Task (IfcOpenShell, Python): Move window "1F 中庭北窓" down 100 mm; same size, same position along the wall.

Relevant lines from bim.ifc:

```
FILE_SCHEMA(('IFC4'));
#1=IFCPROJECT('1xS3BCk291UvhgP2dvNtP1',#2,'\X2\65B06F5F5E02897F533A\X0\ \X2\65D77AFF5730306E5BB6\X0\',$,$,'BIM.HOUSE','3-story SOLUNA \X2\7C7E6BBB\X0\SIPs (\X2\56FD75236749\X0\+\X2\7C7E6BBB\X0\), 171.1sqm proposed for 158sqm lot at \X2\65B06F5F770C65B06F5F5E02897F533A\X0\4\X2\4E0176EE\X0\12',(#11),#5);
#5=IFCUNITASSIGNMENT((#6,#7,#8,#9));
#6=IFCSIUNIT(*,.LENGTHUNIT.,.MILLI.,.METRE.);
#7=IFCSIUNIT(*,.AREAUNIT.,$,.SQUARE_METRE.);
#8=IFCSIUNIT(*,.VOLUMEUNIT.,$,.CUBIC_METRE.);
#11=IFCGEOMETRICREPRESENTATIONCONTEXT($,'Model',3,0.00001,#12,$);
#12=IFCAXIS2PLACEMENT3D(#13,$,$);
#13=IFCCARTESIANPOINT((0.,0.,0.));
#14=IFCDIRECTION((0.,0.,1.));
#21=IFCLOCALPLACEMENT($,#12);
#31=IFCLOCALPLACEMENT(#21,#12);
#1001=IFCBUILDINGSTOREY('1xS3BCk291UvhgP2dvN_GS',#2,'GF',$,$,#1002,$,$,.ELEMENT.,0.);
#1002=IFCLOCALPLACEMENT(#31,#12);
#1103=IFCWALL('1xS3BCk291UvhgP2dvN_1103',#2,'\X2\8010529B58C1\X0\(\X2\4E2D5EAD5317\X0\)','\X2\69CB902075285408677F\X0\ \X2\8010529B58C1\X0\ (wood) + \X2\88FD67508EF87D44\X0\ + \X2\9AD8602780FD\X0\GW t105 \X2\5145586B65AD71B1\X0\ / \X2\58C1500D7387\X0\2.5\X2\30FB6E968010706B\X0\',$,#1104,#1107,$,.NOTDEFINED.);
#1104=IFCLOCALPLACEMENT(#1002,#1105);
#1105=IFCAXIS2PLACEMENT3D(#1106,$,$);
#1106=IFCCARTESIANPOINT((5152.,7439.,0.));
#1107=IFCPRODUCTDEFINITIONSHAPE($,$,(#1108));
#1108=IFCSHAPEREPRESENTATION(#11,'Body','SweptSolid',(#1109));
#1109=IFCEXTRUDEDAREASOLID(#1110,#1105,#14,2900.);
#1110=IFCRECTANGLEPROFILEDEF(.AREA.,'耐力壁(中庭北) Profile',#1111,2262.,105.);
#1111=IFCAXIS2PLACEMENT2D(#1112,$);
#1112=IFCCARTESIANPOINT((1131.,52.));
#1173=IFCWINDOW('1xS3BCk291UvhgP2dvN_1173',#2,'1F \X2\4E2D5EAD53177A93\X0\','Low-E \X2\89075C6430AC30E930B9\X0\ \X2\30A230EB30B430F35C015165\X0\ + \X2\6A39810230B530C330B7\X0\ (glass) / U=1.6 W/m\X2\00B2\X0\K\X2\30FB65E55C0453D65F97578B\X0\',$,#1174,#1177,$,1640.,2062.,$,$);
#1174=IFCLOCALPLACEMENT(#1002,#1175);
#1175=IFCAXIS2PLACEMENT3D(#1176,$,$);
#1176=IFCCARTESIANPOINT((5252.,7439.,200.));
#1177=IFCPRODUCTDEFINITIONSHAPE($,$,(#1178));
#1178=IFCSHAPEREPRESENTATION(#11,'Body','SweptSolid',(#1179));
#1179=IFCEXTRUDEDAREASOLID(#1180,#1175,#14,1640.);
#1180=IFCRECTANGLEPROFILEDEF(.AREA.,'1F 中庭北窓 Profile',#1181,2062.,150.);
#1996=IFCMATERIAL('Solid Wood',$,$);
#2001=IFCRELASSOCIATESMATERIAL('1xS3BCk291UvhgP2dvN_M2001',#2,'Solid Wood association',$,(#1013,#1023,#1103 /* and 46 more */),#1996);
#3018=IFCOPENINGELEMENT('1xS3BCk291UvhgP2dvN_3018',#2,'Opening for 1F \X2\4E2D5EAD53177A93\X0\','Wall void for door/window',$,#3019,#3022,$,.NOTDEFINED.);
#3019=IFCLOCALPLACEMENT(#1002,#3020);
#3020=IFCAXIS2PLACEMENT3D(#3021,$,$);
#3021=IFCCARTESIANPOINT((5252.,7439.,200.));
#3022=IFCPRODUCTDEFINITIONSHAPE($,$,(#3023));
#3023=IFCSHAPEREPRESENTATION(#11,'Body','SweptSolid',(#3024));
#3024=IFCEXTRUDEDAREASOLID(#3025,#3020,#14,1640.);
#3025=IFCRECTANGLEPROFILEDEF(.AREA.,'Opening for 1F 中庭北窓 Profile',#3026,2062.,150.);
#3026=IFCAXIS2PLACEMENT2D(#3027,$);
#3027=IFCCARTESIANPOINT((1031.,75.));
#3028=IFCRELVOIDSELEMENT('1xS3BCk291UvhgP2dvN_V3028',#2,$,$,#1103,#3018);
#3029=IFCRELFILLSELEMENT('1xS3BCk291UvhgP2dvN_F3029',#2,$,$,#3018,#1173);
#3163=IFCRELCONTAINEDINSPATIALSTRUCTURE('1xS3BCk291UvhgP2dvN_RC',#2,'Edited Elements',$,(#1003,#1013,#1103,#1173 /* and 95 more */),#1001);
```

```python
import numpy as np
import ifcopenshell
import ifcopenshell.api.geometry
import ifcopenshell.util.placement
import ifcopenshell.util.unit

model = ifcopenshell.open("bim.ifc")
unit_scale = ifcopenshell.util.unit.calculate_unit_scale(model)

window = model.by_guid("1xS3BCk291UvhgP2dvN_1173")
opening = window.FillsVoids[0].RelatingOpeningElement
dz = -100.0

shift = np.array([0.0, 0.0, dz])
# The window is not placed relative to its opening, so move both.
for product in (opening, window):
    matrix = ifcopenshell.util.placement.get_local_placement(product.ObjectPlacement)
    matrix[:3, 3] += shift
    ifcopenshell.api.geometry.edit_object_placement(model, product=product, matrix=matrix, is_si=False)

print(f"moved by {dz * unit_scale:+.3f} m")

model.write("bim-out.ifc")
```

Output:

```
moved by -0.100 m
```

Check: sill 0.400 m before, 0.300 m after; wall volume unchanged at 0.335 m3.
